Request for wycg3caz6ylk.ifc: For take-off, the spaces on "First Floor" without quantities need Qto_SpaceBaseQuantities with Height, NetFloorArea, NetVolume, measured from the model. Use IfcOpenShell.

First a look at what the model holds.

```python
import ifcopenshell
import ifcopenshell.util.element
import ifcopenshell.util.unit

model = ifcopenshell.open("wycg3caz6ylk.ifc")
print(model.schema)
for unit_type in ("LENGTHUNIT", "AREAUNIT", "VOLUMEUNIT"):
    print(unit_type, ifcopenshell.util.unit.calculate_unit_scale(model, unit_type))
storey = next(s for s in model.by_type("IfcBuildingStorey") if s.Name == "First Floor")
spaces = [e for e in ifcopenshell.util.element.get_decomposition(storey) if e.is_a("IfcSpace")]
for e in sorted(spaces, key=lambda e: e.id()):
    print(e.id(), e.is_a(), e.Name, list(ifcopenshell.util.element.get_psets(e, qtos_only=True)), sep=" | ")
```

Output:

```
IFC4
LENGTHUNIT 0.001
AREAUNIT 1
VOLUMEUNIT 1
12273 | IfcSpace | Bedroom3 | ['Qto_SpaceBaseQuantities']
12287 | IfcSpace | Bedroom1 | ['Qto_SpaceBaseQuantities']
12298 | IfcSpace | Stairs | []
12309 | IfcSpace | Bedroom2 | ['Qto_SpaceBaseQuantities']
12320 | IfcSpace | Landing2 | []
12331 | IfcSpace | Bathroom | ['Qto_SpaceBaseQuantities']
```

```python
import ifcopenshell
import ifcopenshell.api.pset
import ifcopenshell.geom
import ifcopenshell.util.element
import ifcopenshell.util.shape
import ifcopenshell.util.unit

model = ifcopenshell.open("wycg3caz6ylk.ifc")
unit_scale = ifcopenshell.util.unit.calculate_unit_scale(model)
area_scale = ifcopenshell.util.unit.calculate_unit_scale(model, "AREAUNIT")
volume_scale = ifcopenshell.util.unit.calculate_unit_scale(model, "VOLUMEUNIT")
settings = ifcopenshell.geom.settings()

storey = next(s for s in model.by_type("IfcBuildingStorey") if s.Name == "First Floor")
spaces = [e for e in ifcopenshell.util.element.get_decomposition(storey) if e.is_a("IfcSpace")]

for e in sorted(spaces, key=lambda e: e.id()):
    if ifcopenshell.util.element.get_psets(e, qtos_only=True, should_inherit=False):
        continue
    # Geometry comes back in metres, in the element's own axes.
    shape = ifcopenshell.geom.create_shape(settings, e)
    values = {
        "Height": ifcopenshell.util.shape.get_z(shape.geometry) / unit_scale,
        "NetFloorArea": ifcopenshell.util.shape.get_footprint_area(shape.geometry) / area_scale,
        "NetVolume": ifcopenshell.util.shape.get_volume(shape.geometry) / volume_scale,
    }
    qto = ifcopenshell.api.pset.add_qto(model, product=e, name="Qto_SpaceBaseQuantities")
    ifcopenshell.api.pset.edit_qto(model, qto=qto, properties=values)
    print(e.id(), {k: round(v, 3) for k, v in values.items()})

model.write("wycg3caz6ylk_v2.ifc")
```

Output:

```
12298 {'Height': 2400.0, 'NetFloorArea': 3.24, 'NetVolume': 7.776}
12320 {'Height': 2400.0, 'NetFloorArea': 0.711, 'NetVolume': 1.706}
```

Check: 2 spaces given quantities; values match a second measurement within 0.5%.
